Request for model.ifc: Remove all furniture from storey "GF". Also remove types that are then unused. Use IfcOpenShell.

First a look at what the model holds.

```python
import ifcopenshell
import ifcopenshell.util.element

model = ifcopenshell.open("model.ifc")
print(model.schema)
storey = next(s for s in model.by_type("IfcBuildingStorey") if s.Name == "GF")
furniture = [e for e in ifcopenshell.util.element.get_decomposition(storey) if e.is_a("IfcFurnishingElement")]
seen = {}
for e in furniture:
    element_type = ifcopenshell.util.element.get_type(e)
    name = element_type.Name if element_type not in (None, e) else None
    seen[name] = seen.get(name, 0) + 1
for name, count in sorted(seen.items(), key=str):
    print(count, "x", name)
```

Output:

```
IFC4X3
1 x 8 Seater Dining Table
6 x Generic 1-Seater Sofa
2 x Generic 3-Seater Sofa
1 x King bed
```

```python
import ifcopenshell
import ifcopenshell.api.root
import ifcopenshell.util.element

model = ifcopenshell.open("model.ifc")

storey = next(s for s in model.by_type("IfcBuildingStorey") if s.Name == "GF")
furniture = [e for e in ifcopenshell.util.element.get_decomposition(storey) if e.is_a("IfcFurnishingElement")]
types = {ifcopenshell.util.element.get_type(e) for e in furniture} - {None, *furniture}

for e in furniture:
    ifcopenshell.api.root.remove_product(model, product=e)
print(len(furniture), "removed")

unused = [t for t in types if not ifcopenshell.util.element.get_types(t)]
for t in unused:
    ifcopenshell.api.root.remove_product(model, product=t)
print(len(unused), "unused types removed")

model.write("model_updated.ifc")
```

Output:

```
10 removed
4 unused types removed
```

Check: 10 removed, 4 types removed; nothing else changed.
